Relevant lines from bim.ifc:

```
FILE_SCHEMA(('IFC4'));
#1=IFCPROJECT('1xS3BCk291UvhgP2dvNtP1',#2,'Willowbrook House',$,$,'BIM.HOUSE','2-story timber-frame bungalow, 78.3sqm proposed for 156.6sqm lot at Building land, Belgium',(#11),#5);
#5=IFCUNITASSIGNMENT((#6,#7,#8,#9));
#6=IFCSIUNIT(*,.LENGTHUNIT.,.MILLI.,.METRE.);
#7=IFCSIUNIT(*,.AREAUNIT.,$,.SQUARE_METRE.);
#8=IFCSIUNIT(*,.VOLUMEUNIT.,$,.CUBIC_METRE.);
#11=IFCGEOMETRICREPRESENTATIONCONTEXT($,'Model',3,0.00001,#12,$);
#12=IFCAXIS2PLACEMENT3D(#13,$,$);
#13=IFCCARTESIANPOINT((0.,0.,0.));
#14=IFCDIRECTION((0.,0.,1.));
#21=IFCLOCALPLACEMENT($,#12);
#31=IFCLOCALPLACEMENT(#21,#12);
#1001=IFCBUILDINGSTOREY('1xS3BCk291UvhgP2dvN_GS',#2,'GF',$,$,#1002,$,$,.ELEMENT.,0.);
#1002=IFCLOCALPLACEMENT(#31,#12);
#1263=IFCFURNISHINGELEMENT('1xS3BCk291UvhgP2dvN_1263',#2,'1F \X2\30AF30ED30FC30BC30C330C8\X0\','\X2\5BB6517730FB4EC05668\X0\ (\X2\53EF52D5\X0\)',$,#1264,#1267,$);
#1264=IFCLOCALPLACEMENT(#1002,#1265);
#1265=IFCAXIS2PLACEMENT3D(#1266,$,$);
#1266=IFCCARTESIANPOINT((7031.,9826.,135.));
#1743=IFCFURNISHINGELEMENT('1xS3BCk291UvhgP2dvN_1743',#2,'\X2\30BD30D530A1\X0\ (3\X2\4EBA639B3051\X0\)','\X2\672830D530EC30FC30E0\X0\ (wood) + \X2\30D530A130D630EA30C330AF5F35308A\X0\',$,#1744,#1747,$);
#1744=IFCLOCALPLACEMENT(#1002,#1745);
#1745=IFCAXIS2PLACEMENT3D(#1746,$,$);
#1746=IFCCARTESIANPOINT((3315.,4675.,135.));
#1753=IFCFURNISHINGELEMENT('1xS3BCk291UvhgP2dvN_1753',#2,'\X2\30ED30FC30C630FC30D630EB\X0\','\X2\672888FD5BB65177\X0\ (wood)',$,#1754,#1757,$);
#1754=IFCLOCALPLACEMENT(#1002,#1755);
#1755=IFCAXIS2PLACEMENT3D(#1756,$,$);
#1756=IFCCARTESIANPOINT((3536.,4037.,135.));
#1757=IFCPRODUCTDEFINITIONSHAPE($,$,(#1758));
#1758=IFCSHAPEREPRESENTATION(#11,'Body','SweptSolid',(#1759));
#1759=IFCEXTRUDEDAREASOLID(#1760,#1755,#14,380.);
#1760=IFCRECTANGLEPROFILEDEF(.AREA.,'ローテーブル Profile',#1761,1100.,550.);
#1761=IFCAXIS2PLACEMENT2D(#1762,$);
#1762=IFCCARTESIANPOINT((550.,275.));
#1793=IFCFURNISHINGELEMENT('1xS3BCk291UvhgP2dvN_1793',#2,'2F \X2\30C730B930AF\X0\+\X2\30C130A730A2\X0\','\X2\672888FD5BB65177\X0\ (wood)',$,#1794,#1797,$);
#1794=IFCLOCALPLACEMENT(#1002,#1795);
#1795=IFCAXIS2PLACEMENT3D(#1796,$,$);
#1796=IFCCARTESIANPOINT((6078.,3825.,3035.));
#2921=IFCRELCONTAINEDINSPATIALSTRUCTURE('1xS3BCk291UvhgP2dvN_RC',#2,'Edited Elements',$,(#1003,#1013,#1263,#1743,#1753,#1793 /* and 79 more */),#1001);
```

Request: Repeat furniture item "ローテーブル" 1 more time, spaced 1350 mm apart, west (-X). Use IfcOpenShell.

```python
import numpy as np
import ifcopenshell
import ifcopenshell.api.geometry
import ifcopenshell.api.root
import ifcopenshell.util.element
import ifcopenshell.util.placement

model = ifcopenshell.open("bim.ifc")


def reuse_history(source, copy):
    """copy_class also copies each property set's owner history, people and application; keep the originals."""
    for rel in copy.IsDefinedBy:
        if rel.is_a("IfcRelDefinesByProperties") and (history := rel.RelatingPropertyDefinition.OwnerHistory):
            rel.RelatingPropertyDefinition.OwnerHistory = source.OwnerHistory
            ifcopenshell.util.element.remove_deep2(model, history)


source = model.by_guid("1xS3BCk291UvhgP2dvN_1753")
base = ifcopenshell.util.placement.get_local_placement(source.ObjectPlacement)
step = np.array([-1.0, 0.0, 0.0]) * 1350.0

for i in range(1, 2):
    copy = ifcopenshell.api.root.copy_class(model, product=source)
    copy.Representation = ifcopenshell.util.element.copy_deep(
        model, source.Representation, exclude=["IfcGeometricRepresentationContext", "IfcRepresentationMap"]
    )
    reuse_history(source, copy)
    matrix = base.copy()
    matrix[:3, 3] += i * step
    print("added at", matrix[:3, 3].round(3) + 0.0)
    ifcopenshell.api.geometry.edit_object_placement(model, product=copy, matrix=matrix, is_si=False)

model.write("bim_rev.ifc")
```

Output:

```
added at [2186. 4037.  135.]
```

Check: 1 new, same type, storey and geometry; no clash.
